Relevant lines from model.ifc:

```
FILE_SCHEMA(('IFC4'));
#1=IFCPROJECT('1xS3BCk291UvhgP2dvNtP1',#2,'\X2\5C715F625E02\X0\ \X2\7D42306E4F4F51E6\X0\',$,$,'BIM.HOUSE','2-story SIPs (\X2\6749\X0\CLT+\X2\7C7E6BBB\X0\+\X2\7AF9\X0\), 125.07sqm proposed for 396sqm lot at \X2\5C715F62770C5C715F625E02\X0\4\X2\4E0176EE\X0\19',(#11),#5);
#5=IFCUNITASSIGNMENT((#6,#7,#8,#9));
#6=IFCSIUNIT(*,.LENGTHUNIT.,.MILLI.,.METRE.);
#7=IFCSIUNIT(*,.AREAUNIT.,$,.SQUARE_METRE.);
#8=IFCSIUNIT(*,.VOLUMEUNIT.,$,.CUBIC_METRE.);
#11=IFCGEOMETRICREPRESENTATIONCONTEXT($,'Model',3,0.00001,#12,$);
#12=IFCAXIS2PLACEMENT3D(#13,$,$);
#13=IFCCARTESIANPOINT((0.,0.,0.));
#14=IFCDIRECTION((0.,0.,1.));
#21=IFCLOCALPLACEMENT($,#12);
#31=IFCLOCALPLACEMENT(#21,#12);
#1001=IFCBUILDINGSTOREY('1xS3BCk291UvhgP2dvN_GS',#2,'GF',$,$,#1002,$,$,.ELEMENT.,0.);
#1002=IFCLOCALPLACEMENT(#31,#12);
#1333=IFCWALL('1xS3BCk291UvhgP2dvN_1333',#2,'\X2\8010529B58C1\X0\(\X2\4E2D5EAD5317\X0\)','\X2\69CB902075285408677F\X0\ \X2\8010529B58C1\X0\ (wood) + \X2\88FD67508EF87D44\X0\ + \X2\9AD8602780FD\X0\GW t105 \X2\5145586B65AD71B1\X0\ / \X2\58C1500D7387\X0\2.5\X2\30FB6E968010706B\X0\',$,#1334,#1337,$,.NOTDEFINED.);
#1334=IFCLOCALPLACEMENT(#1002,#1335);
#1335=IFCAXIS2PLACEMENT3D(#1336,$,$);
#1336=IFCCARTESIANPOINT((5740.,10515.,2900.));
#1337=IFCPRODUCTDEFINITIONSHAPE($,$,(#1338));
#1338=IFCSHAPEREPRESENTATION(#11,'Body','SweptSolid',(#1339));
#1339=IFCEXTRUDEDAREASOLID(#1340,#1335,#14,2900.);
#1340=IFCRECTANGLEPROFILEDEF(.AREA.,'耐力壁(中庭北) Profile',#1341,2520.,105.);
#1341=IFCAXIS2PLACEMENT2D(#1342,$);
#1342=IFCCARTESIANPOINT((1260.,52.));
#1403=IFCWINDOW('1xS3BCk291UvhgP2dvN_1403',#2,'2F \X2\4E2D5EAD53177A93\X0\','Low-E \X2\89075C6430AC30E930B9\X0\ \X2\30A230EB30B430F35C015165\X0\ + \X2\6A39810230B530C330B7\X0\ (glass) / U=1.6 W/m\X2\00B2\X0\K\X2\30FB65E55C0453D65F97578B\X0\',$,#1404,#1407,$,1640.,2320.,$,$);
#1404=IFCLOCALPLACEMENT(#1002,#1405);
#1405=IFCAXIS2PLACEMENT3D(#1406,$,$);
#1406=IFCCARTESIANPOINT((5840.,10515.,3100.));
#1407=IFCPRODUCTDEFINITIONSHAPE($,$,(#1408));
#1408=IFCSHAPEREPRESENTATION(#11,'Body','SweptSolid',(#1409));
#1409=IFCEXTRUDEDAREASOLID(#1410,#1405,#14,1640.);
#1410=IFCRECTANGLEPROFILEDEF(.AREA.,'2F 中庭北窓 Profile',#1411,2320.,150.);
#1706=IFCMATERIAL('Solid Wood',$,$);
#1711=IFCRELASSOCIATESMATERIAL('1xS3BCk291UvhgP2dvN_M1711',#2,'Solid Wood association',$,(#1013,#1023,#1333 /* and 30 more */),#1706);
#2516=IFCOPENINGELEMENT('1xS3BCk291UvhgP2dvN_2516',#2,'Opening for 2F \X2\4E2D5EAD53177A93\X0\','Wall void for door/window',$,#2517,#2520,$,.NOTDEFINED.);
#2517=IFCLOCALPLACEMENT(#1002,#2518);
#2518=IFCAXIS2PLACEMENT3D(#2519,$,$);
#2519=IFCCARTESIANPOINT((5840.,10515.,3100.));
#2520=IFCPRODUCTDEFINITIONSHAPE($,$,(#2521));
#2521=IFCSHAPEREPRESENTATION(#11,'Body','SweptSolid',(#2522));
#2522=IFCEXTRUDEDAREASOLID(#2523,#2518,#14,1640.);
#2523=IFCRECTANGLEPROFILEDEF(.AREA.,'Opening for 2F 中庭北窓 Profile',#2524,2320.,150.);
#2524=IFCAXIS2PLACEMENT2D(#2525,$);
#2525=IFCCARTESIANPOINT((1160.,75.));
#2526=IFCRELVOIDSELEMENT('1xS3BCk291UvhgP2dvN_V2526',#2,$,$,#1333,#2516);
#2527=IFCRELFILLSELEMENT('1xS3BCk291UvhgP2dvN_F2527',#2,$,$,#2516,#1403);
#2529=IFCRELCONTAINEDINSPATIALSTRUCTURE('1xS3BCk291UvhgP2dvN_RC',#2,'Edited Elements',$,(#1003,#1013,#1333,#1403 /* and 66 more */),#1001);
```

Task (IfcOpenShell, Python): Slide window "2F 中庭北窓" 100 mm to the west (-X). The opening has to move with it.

```python
import ifcopenshell
import ifcopenshell.api.geometry
import ifcopenshell.util.placement

model = ifcopenshell.open("model.ifc")

window = model.by_guid("1xS3BCk291UvhgP2dvN_1403")
opening = window.FillsVoids[0].RelatingOpeningElement
wall = opening.VoidsElements[0].RelatingBuildingElement

wall_matrix = ifcopenshell.util.placement.get_local_placement(wall.ObjectPlacement)
shift = wall_matrix[:3, 0] * -100.0
before = ifcopenshell.util.placement.get_local_placement(window.ObjectPlacement)[:3, 3].copy()

# The window is not placed relative to its opening, so move both.
for product in (opening, window):
    matrix = ifcopenshell.util.placement.get_local_placement(product.ObjectPlacement)
    matrix[:3, 3] += shift
    ifcopenshell.api.geometry.edit_object_placement(model, product=product, matrix=matrix, is_si=False)

after = ifcopenshell.util.placement.get_local_placement(window.ObjectPlacement)[:3, 3]
print("window moved by", (after - before).round(3) + 0.0)

model.write("model_rev.ifc")
```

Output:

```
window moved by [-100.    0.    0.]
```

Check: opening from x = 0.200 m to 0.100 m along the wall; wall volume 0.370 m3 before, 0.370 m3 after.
